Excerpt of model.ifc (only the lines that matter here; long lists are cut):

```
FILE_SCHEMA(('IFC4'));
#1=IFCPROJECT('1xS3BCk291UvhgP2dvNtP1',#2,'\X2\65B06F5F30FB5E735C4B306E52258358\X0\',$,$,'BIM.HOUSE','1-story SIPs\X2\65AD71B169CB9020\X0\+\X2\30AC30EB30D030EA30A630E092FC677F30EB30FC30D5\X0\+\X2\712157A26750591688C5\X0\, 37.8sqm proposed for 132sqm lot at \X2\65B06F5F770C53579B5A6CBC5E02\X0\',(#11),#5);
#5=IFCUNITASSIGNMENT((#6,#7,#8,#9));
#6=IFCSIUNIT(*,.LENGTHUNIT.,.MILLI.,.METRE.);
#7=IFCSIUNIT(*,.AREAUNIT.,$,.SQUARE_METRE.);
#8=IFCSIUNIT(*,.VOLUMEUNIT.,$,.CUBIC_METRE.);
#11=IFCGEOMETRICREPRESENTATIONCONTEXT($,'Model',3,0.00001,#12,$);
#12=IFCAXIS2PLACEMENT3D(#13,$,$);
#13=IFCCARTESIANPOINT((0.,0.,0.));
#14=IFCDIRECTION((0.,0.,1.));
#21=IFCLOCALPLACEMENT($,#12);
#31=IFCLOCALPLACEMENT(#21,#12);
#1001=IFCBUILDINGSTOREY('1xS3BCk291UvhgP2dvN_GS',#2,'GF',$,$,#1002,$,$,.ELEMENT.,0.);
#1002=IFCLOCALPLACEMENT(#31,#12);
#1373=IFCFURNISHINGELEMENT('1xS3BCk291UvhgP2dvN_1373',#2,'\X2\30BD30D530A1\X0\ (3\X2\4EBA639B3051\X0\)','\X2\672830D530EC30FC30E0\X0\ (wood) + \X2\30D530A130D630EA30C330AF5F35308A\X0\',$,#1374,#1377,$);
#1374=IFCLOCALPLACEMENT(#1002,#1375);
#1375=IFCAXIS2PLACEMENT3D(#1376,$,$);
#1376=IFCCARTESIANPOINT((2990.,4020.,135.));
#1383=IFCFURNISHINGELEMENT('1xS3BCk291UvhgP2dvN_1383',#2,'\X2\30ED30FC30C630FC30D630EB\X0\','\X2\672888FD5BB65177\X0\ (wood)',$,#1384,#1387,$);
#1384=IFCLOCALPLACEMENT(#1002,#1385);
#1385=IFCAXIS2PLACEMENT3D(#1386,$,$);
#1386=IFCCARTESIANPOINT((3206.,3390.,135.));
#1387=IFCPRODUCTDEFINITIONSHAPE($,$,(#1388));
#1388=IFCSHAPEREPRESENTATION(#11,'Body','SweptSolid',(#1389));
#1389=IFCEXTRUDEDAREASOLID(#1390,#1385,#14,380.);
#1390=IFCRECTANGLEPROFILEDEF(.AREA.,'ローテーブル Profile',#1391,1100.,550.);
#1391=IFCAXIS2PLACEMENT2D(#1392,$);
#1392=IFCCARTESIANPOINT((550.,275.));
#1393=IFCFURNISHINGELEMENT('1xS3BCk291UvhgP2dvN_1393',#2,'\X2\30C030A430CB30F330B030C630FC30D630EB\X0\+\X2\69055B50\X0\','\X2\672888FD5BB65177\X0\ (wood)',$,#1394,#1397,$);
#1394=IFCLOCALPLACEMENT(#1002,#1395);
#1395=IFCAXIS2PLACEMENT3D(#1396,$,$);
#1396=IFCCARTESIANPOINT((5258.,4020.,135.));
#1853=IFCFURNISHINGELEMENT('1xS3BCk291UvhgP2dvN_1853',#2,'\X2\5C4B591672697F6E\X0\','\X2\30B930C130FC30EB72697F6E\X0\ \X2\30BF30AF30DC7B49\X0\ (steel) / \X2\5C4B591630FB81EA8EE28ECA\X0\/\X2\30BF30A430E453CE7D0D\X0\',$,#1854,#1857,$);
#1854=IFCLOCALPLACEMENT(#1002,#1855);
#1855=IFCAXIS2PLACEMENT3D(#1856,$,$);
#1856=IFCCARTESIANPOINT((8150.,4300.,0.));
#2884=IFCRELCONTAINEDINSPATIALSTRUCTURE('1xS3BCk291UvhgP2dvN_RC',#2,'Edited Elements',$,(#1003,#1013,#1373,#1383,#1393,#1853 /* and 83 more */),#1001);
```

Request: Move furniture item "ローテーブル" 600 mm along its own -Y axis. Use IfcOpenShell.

```python
import ifcopenshell
import ifcopenshell.api.geometry
import ifcopenshell.util.placement

model = ifcopenshell.open("model.ifc")

item = model.by_guid("1xS3BCk291UvhgP2dvN_1383")
matrix = ifcopenshell.util.placement.get_local_placement(item.ObjectPlacement)
matrix[:3, 3] -= matrix[:3, 1] * 600.0
ifcopenshell.api.geometry.edit_object_placement(model, product=item, matrix=matrix, is_si=False)

print(ifcopenshell.util.placement.get_local_placement(item.ObjectPlacement).round(3) + 0.0)

model.write("model_v2.ifc")
```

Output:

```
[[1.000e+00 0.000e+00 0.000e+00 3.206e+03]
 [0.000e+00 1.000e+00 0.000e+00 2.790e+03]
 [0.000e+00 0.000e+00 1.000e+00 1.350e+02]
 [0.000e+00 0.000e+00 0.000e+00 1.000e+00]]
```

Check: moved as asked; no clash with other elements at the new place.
